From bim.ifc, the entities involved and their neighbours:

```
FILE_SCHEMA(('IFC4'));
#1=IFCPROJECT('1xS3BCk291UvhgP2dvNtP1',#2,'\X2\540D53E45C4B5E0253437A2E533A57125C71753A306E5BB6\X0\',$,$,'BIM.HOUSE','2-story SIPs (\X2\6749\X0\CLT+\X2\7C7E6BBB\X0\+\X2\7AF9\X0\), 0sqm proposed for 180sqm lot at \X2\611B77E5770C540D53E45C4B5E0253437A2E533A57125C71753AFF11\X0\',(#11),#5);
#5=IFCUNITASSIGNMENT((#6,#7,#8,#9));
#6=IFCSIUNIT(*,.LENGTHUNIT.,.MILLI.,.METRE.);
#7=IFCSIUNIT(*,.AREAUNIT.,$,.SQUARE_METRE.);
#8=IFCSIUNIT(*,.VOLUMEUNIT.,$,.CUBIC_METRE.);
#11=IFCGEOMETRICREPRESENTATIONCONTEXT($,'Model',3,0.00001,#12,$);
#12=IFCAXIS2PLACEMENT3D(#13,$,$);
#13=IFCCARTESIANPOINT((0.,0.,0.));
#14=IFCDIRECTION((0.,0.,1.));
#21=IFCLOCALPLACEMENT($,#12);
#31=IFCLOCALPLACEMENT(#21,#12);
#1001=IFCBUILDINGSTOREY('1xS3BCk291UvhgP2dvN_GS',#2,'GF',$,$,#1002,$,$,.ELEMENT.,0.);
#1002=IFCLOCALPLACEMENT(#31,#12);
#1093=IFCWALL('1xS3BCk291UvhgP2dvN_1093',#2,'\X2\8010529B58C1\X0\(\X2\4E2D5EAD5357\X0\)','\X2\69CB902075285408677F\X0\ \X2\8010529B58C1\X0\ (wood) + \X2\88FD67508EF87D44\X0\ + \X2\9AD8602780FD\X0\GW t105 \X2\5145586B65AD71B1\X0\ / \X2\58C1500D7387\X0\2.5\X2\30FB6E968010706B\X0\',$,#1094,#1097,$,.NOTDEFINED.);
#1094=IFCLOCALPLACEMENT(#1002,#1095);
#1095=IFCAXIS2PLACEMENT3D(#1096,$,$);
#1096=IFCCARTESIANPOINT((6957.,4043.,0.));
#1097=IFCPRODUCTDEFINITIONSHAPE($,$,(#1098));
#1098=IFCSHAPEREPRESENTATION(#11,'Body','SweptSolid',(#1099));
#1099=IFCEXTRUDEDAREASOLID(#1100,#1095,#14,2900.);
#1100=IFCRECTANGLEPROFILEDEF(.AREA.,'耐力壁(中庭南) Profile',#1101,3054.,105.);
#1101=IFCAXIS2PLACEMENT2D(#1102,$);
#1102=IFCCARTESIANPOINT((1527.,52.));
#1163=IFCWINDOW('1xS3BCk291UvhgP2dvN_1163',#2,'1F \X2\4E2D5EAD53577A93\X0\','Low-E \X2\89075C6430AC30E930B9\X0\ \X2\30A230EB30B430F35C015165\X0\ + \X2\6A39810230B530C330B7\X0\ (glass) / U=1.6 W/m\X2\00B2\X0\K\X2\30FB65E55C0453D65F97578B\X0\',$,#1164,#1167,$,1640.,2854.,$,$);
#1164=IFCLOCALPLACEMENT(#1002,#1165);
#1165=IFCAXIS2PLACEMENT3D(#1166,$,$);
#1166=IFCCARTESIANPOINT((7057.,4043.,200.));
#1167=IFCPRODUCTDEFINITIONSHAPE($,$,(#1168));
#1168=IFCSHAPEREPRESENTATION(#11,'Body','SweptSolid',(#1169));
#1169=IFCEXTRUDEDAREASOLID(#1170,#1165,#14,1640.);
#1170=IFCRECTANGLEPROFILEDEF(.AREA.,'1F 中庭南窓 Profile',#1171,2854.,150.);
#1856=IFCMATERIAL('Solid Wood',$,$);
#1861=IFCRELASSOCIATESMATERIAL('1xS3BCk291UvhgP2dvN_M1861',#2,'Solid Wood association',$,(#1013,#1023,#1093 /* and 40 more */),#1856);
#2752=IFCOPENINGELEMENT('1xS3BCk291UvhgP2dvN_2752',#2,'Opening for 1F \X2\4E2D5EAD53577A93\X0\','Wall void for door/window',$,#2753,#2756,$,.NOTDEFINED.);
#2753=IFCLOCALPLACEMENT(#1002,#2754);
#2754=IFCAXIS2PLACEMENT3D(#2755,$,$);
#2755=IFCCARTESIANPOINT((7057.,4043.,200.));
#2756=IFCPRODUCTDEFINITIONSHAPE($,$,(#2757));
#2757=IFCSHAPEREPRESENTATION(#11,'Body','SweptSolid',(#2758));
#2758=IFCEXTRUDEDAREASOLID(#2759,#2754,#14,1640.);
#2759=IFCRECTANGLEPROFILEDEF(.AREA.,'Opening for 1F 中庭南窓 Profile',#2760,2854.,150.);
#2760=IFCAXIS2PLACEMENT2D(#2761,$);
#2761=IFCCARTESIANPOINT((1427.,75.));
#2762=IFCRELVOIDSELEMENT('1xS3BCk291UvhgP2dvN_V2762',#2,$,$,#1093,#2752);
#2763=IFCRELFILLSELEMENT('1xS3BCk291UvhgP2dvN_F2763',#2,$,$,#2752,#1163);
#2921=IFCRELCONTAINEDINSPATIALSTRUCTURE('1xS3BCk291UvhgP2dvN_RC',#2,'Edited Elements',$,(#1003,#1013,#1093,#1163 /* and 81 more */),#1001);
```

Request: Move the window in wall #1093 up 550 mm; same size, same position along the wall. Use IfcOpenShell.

```python
import numpy as np
import ifcopenshell
import ifcopenshell.api.geometry
import ifcopenshell.util.placement
import ifcopenshell.util.unit

model = ifcopenshell.open("bim.ifc")
unit_scale = ifcopenshell.util.unit.calculate_unit_scale(model)

window = model.by_id(1163)
opening = window.FillsVoids[0].RelatingOpeningElement
dz = 0.55 / unit_scale

shift = np.array([0.0, 0.0, dz])
# The window is not placed relative to its opening, so move both.
for product in (opening, window):
    matrix = ifcopenshell.util.placement.get_local_placement(product.ObjectPlacement)
    matrix[:3, 3] += shift
    ifcopenshell.api.geometry.edit_object_placement(model, product=product, matrix=matrix, is_si=False)

print(f"moved by {dz * unit_scale:+.3f} m")

model.write("bim_v2.ifc")
```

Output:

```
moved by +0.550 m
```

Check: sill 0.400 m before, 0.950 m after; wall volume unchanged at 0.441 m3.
